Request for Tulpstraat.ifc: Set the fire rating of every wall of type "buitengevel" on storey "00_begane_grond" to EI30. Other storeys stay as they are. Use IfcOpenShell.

First a look at what the model holds.

```python
import ifcopenshell
import ifcopenshell.util.element

model = ifcopenshell.open("Tulpstraat.ifc")
print(model.schema)
storey = next(s for s in model.by_type("IfcBuildingStorey") if s.Name == "00_begane_grond")
walls = [e for e in ifcopenshell.util.element.get_decomposition(storey) if e.is_a("IfcWall")]
seen = {}
for e in walls:
    element_type = ifcopenshell.util.element.get_type(e)
    key = (element_type.Name if element_type != e and element_type else None, ifcopenshell.util.element.get_pset(e, "Pset_WallCommon", "FireRating"))
    seen[key] = seen.get(key, 0) + 1
for (name, value), count in sorted(seen.items(), key=str):
    print(count, "x", name, "|", value)
```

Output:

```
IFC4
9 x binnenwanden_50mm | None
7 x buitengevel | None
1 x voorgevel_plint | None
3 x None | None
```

```python
import ifcopenshell
import ifcopenshell.api.pset
import ifcopenshell.util.element

model = ifcopenshell.open("Tulpstraat.ifc")

storey = next(s for s in model.by_type("IfcBuildingStorey") if s.Name == "00_begane_grond")
walls = [e for e in ifcopenshell.util.element.get_decomposition(storey) if e.is_a("IfcWall")]

count = 0
for e in walls:
    element_type = ifcopenshell.util.element.get_type(e)
    if element_type in (None, e) or element_type.Name != "buitengevel":
        continue
    # add_pset returns the element's existing set when there is one.
    pset = ifcopenshell.api.pset.add_pset(model, product=e, name="Pset_WallCommon")
    ifcopenshell.api.pset.edit_pset(model, pset=pset, properties={"FireRating": "EI30"})
    count += 1

print(count, "walls updated")

model.write("Tulpstraat_edited.ifc")
```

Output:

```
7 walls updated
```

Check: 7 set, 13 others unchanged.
